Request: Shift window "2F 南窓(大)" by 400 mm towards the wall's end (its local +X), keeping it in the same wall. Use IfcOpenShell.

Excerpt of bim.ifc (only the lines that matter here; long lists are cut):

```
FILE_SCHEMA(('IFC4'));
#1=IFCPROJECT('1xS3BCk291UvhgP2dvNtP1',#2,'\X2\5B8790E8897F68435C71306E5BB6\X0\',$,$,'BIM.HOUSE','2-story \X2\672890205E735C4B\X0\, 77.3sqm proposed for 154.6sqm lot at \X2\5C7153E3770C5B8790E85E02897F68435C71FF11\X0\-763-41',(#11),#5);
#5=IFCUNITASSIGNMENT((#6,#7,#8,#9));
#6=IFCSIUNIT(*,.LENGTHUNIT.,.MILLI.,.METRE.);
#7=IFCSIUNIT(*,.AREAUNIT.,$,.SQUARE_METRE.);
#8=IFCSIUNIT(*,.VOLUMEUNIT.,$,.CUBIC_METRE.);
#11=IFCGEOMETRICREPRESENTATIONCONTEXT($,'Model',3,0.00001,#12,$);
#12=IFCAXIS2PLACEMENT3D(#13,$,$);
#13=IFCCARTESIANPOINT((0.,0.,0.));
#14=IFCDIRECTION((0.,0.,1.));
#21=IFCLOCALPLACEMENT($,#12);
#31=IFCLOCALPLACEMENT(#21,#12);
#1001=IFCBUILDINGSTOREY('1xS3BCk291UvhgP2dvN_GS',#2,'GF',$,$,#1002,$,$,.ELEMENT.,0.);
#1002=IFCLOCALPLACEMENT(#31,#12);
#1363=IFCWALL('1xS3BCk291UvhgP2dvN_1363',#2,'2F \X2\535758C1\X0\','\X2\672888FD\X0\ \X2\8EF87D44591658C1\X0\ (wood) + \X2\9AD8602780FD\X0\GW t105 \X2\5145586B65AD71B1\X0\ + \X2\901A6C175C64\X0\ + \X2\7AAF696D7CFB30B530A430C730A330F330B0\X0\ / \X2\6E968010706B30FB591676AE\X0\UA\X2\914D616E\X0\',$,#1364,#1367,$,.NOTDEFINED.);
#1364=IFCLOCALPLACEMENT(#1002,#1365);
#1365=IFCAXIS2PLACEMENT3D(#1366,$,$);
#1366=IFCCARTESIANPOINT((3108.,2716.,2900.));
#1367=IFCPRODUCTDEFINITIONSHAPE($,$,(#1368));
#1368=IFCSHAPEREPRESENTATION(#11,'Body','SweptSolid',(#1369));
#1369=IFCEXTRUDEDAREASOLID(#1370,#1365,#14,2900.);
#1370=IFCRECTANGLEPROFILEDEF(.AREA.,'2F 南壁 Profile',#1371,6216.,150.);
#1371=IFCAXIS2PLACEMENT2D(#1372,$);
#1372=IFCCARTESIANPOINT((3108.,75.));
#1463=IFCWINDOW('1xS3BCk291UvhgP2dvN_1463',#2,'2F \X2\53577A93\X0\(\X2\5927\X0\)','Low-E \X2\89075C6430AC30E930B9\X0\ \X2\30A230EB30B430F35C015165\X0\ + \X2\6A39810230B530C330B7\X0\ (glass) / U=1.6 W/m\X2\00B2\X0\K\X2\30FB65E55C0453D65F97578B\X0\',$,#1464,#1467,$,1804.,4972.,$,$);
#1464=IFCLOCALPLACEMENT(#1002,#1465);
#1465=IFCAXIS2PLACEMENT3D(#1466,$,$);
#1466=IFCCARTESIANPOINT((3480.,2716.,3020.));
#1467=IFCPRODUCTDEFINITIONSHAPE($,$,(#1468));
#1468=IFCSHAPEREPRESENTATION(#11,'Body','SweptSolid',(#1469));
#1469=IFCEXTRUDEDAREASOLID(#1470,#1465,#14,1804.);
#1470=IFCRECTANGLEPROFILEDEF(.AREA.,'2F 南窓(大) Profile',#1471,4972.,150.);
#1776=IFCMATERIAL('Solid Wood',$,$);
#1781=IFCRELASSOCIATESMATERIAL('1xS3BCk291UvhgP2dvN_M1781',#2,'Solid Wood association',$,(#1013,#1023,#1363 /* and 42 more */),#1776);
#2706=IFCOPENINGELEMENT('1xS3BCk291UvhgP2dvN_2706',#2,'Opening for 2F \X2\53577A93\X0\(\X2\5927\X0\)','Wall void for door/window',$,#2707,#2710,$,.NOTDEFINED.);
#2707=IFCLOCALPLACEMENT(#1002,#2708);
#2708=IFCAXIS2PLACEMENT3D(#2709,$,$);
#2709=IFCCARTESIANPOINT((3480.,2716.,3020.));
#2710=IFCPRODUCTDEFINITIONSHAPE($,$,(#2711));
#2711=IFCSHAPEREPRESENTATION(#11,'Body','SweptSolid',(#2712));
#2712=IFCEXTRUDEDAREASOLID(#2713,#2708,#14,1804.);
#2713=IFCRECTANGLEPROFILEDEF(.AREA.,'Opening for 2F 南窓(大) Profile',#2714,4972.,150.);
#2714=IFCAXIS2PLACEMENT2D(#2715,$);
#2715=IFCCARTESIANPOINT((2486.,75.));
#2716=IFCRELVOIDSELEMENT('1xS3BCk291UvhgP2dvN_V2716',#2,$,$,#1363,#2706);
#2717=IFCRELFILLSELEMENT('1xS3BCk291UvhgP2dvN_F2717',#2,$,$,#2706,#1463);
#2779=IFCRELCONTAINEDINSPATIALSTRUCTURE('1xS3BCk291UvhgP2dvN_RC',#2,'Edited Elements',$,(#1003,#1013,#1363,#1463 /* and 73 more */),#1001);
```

```python
import ifcopenshell
import ifcopenshell.api.geometry
import ifcopenshell.util.placement

model = ifcopenshell.open("bim.ifc")

window = model.by_guid("1xS3BCk291UvhgP2dvN_1463")
opening = window.FillsVoids[0].RelatingOpeningElement
wall = opening.VoidsElements[0].RelatingBuildingElement

wall_matrix = ifcopenshell.util.placement.get_local_placement(wall.ObjectPlacement)
shift = wall_matrix[:3, 0] * 400.0
before = ifcopenshell.util.placement.get_local_placement(window.ObjectPlacement)[:3, 3].copy()

# The window is not placed relative to its opening, so move both.
for product in (opening, window):
    matrix = ifcopenshell.util.placement.get_local_placement(product.ObjectPlacement)
    matrix[:3, 3] += shift
    ifcopenshell.api.geometry.edit_object_placement(model, product=product, matrix=matrix, is_si=False)

after = ifcopenshell.util.placement.get_local_placement(window.ObjectPlacement)[:3, 3]
print("window moved by", (after - before).round(3) + 0.0)

model.write("bim_updated.ifc")
```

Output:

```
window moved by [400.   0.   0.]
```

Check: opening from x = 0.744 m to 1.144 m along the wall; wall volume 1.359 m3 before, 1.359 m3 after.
